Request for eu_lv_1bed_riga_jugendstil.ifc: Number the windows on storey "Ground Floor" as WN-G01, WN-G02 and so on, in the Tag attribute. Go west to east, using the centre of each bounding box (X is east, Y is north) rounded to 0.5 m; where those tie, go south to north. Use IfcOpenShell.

First a look at what the model holds.

```python
import ifcopenshell
import ifcopenshell.util.element
import ifcopenshell.util.placement

model = ifcopenshell.open("eu_lv_1bed_riga_jugendstil.ifc")
print(model.schema)
storey = next(s for s in model.by_type("IfcBuildingStorey") if s.Name == "Ground Floor")
windows = [e for e in ifcopenshell.util.element.get_decomposition(storey) if e.is_a("IfcWindow")]
for e in sorted(windows, key=lambda e: e.id()):
    origin = ifcopenshell.util.placement.get_local_placement(e.ObjectPlacement)[:3, 3]
    print(e.id(), e.Tag, e.Name, origin.round(2) + 0.0, sep=" | ")
```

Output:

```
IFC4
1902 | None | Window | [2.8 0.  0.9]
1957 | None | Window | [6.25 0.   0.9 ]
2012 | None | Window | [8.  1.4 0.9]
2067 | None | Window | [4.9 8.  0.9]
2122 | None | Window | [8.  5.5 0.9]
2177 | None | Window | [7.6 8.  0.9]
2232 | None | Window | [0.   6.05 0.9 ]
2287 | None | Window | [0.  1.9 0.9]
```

```python
import ifcopenshell
import ifcopenshell.geom
import ifcopenshell.util.element
import ifcopenshell.util.shape

model = ifcopenshell.open("eu_lv_1bed_riga_jugendstil.ifc")
settings = ifcopenshell.geom.settings()
settings.set("use-world-coords", True)


def centre(element):
    shape = ifcopenshell.geom.create_shape(settings, element)
    return ifcopenshell.util.shape.get_bbox_centroid(shape.geometry)


storey = next(s for s in model.by_type("IfcBuildingStorey") if s.Name == "Ground Floor")
windows = [e for e in ifcopenshell.util.element.get_decomposition(storey) if e.is_a("IfcWindow")]

# Insertion points can sit at a corner or the storey origin, so sort by the geometry (in metres).
centres = {e: centre(e) for e in windows}
windows.sort(key=lambda e: (round(centres[e][0] / 0.5), centres[e][1]))

for i, e in enumerate(windows, start=1):
    number = f"WN-G{i:02d}"
    e.Tag = number
    print(e.id(), number)

model.write("eu_lv_1bed_riga_jugendstil_rev.ifc")
```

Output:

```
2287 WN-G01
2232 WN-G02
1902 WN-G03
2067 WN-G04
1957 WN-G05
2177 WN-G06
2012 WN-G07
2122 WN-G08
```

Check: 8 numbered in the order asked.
